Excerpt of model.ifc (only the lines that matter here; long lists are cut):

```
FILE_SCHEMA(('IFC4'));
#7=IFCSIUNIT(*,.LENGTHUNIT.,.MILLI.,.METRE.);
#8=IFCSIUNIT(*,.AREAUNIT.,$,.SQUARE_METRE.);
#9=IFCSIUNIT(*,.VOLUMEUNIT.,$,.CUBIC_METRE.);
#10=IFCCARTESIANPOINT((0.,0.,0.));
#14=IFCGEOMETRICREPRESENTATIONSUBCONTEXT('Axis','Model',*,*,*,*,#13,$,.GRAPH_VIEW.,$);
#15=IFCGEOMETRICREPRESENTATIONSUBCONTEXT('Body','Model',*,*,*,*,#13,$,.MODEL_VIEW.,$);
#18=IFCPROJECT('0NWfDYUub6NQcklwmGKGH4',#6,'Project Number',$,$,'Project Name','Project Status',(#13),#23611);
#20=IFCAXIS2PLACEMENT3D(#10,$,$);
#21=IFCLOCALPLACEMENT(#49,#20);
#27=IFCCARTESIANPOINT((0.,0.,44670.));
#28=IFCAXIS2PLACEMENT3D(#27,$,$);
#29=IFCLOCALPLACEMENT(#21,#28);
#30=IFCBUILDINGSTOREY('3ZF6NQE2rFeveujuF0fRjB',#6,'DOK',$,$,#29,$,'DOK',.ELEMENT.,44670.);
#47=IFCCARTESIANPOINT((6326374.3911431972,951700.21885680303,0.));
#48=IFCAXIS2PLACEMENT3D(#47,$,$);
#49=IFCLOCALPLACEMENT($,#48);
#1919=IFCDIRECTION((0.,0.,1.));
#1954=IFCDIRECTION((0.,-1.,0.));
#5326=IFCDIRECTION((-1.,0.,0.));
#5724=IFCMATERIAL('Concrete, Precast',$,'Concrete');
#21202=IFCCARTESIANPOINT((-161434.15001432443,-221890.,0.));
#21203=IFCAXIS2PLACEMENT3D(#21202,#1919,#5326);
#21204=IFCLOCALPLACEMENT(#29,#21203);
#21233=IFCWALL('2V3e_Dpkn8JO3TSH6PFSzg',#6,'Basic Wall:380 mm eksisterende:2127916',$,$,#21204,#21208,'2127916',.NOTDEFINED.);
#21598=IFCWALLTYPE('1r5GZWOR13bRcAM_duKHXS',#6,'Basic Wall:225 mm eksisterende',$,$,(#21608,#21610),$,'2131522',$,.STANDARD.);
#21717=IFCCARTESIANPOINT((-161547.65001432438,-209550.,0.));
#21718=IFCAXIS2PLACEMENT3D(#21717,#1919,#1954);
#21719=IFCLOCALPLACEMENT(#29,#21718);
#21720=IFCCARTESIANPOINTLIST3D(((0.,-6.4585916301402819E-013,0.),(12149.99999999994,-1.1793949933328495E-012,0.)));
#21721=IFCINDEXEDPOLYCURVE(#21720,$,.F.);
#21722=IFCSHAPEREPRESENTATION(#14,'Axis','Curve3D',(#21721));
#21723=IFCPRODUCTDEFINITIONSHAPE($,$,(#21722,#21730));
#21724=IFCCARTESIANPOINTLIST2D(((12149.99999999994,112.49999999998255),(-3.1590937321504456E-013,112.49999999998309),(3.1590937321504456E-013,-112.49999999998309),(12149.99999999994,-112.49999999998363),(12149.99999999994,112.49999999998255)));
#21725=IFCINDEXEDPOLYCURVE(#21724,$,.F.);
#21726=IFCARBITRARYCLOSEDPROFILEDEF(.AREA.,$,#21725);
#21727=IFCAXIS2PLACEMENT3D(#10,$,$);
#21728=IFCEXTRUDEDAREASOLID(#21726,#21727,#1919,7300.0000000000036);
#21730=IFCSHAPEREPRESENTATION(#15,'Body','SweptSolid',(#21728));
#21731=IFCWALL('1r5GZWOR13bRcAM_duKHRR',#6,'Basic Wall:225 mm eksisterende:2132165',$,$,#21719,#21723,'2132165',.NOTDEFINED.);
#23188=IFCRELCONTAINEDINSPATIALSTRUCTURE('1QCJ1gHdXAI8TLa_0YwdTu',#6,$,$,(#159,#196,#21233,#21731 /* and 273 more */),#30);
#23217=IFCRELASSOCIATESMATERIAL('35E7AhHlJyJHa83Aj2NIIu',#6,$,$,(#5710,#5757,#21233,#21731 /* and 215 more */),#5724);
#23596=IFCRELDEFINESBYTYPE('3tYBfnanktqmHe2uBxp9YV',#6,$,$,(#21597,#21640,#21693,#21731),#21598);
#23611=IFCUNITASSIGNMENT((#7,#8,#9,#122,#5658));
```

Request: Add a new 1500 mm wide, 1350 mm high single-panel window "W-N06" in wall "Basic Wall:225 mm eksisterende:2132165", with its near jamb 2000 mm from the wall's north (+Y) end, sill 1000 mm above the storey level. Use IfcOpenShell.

```python
import numpy as np
import ifcopenshell
import ifcopenshell.api.feature
import ifcopenshell.api.geometry
import ifcopenshell.api.root
import ifcopenshell.api.spatial
import ifcopenshell.geom
import ifcopenshell.util.element
import ifcopenshell.util.placement
import ifcopenshell.util.representation
import ifcopenshell.util.shape
import ifcopenshell.util.unit

model = ifcopenshell.open("model.ifc")
unit_scale = ifcopenshell.util.unit.calculate_unit_scale(model)
settings = ifcopenshell.geom.settings()


def volume(element):
    """Net volume in cubic metres, openings subtracted."""
    shape = ifcopenshell.geom.create_shape(settings, element)
    return ifcopenshell.util.shape.get_volume(shape.geometry)


wall = model.by_id(21731)
storey = ifcopenshell.util.element.get_container(wall, ifc_class="IfcBuildingStorey")
context = ifcopenshell.util.representation.get_context(model, "Model", "Body", "MODEL_VIEW")
before = volume(wall)

width, height, from_end, sill = 1.5, 1.35, 2, 1  # metres

# The wall runs along its own X axis, and the end named is its -X end.
wall_shape = ifcopenshell.geom.create_shape(settings, wall)
x, y, z = ifcopenshell.util.shape.get_vertices(wall_shape.geometry).T
start = x.min() + from_end
face, thickness = float(y.min()), float(y.max() - y.min())
wall_matrix = ifcopenshell.util.placement.get_local_placement(wall.ObjectPlacement)
level = ifcopenshell.util.placement.get_local_placement(storey.ObjectPlacement)[2, 3]


def in_wall(x, y):
    """Placement at x, y metres in the wall's axes, at sill height."""
    matrix = wall_matrix.copy()
    matrix[:, 3] = wall_matrix @ np.array([x / unit_scale, y / unit_scale, 0.0, 1.0])
    matrix[2, 3] = level + sill / unit_scale
    return matrix


# Opening: a box that overshoots both wall faces by 50 mm.
opening = ifcopenshell.api.root.create_entity(model, ifc_class="IfcOpeningElement", predefined_type="OPENING")
box = ifcopenshell.api.geometry.add_wall_representation(
    model, context=context, length=width, height=height, thickness=thickness + 0.1
)
ifcopenshell.api.geometry.assign_representation(model, product=opening, representation=box)
ifcopenshell.api.geometry.edit_object_placement(model, product=opening, matrix=in_wall(start, face - 0.05), is_si=False)
ifcopenshell.api.feature.add_feature(model, feature=opening, element=wall)

window = ifcopenshell.api.root.create_entity(model, ifc_class="IfcWindow", name="W-N06", predefined_type="WINDOW")
window.OverallWidth, window.OverallHeight = width / unit_scale, height / unit_scale
window.PartitioningType = "SINGLE_PANEL"
body = ifcopenshell.api.geometry.add_window_representation(
    model,
    context=context,
    overall_width=window.OverallWidth,
    overall_height=window.OverallHeight,
    partition_type="SINGLE_PANEL",
)
ifcopenshell.api.geometry.assign_representation(model, product=window, representation=body)
ifcopenshell.api.spatial.assign_container(model, products=[window], relating_structure=storey)
ifcopenshell.api.feature.add_filling(model, opening=opening, element=window)

# Centre the window in the wall's thickness.
ifcopenshell.api.geometry.edit_object_placement(model, product=window, matrix=in_wall(start, face), is_si=False)
window_shape = ifcopenshell.geom.create_shape(settings, window)
depth = ifcopenshell.util.shape.get_vertices(window_shape.geometry)[:, 1]
offset = face + thickness / 2 - (depth.min() + depth.max()) / 2
ifcopenshell.api.geometry.edit_object_placement(model, product=window, matrix=in_wall(start, offset), is_si=False)

after = volume(wall)

print(f"wall volume {before:.3f} -> {after:.3f} m3")

model.write("model-out.ifc")
```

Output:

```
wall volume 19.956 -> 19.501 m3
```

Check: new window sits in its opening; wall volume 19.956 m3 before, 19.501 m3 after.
